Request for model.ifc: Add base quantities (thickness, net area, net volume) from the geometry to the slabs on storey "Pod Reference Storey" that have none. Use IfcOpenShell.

First a look at what the model holds.

```python
import ifcopenshell
import ifcopenshell.util.element
import ifcopenshell.util.unit

model = ifcopenshell.open("model.ifc")
print(model.schema)
for unit_type in ("LENGTHUNIT", "AREAUNIT", "VOLUMEUNIT"):
    print(unit_type, ifcopenshell.util.unit.calculate_unit_scale(model, unit_type))
storey = next(s for s in model.by_type("IfcBuildingStorey") if s.Name == "Pod Reference Storey")
slabs = [e for e in ifcopenshell.util.element.get_decomposition(storey) if e.is_a("IfcSlab")]
for e in sorted(slabs, key=lambda e: e.id()):
    print(e.id(), e.is_a(), e.Name, list(ifcopenshell.util.element.get_psets(e, qtos_only=True)), sep=" | ")
```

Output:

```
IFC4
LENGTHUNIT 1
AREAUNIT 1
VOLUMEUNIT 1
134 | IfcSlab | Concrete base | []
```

```python
import ifcopenshell
import ifcopenshell.api.pset
import ifcopenshell.geom
import ifcopenshell.util.element
import ifcopenshell.util.shape
import ifcopenshell.util.unit

model = ifcopenshell.open("model.ifc")
unit_scale = ifcopenshell.util.unit.calculate_unit_scale(model)
area_scale = ifcopenshell.util.unit.calculate_unit_scale(model, "AREAUNIT")
volume_scale = ifcopenshell.util.unit.calculate_unit_scale(model, "VOLUMEUNIT")
settings = ifcopenshell.geom.settings()

storey = next(s for s in model.by_type("IfcBuildingStorey") if s.Name == "Pod Reference Storey")
slabs = [e for e in ifcopenshell.util.element.get_decomposition(storey) if e.is_a("IfcSlab")]

for e in sorted(slabs, key=lambda e: e.id()):
    if ifcopenshell.util.element.get_psets(e, qtos_only=True, should_inherit=False):
        continue
    # Geometry comes back in metres, in the element's own axes.
    shape = ifcopenshell.geom.create_shape(settings, e)
    values = {
        "Width": ifcopenshell.util.shape.get_z(shape.geometry) / unit_scale,
        "NetArea": ifcopenshell.util.shape.get_footprint_area(shape.geometry) / area_scale,
        "NetVolume": ifcopenshell.util.shape.get_volume(shape.geometry) / volume_scale,
    }
    qto = ifcopenshell.api.pset.add_qto(model, product=e, name="Qto_SlabBaseQuantities")
    ifcopenshell.api.pset.edit_qto(model, qto=qto, properties=values)
    print(e.id(), {k: round(v, 3) for k, v in values.items()})

model.write("model_edited.ifc")
```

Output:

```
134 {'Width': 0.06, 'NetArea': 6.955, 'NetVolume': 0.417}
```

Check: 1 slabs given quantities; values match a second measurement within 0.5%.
